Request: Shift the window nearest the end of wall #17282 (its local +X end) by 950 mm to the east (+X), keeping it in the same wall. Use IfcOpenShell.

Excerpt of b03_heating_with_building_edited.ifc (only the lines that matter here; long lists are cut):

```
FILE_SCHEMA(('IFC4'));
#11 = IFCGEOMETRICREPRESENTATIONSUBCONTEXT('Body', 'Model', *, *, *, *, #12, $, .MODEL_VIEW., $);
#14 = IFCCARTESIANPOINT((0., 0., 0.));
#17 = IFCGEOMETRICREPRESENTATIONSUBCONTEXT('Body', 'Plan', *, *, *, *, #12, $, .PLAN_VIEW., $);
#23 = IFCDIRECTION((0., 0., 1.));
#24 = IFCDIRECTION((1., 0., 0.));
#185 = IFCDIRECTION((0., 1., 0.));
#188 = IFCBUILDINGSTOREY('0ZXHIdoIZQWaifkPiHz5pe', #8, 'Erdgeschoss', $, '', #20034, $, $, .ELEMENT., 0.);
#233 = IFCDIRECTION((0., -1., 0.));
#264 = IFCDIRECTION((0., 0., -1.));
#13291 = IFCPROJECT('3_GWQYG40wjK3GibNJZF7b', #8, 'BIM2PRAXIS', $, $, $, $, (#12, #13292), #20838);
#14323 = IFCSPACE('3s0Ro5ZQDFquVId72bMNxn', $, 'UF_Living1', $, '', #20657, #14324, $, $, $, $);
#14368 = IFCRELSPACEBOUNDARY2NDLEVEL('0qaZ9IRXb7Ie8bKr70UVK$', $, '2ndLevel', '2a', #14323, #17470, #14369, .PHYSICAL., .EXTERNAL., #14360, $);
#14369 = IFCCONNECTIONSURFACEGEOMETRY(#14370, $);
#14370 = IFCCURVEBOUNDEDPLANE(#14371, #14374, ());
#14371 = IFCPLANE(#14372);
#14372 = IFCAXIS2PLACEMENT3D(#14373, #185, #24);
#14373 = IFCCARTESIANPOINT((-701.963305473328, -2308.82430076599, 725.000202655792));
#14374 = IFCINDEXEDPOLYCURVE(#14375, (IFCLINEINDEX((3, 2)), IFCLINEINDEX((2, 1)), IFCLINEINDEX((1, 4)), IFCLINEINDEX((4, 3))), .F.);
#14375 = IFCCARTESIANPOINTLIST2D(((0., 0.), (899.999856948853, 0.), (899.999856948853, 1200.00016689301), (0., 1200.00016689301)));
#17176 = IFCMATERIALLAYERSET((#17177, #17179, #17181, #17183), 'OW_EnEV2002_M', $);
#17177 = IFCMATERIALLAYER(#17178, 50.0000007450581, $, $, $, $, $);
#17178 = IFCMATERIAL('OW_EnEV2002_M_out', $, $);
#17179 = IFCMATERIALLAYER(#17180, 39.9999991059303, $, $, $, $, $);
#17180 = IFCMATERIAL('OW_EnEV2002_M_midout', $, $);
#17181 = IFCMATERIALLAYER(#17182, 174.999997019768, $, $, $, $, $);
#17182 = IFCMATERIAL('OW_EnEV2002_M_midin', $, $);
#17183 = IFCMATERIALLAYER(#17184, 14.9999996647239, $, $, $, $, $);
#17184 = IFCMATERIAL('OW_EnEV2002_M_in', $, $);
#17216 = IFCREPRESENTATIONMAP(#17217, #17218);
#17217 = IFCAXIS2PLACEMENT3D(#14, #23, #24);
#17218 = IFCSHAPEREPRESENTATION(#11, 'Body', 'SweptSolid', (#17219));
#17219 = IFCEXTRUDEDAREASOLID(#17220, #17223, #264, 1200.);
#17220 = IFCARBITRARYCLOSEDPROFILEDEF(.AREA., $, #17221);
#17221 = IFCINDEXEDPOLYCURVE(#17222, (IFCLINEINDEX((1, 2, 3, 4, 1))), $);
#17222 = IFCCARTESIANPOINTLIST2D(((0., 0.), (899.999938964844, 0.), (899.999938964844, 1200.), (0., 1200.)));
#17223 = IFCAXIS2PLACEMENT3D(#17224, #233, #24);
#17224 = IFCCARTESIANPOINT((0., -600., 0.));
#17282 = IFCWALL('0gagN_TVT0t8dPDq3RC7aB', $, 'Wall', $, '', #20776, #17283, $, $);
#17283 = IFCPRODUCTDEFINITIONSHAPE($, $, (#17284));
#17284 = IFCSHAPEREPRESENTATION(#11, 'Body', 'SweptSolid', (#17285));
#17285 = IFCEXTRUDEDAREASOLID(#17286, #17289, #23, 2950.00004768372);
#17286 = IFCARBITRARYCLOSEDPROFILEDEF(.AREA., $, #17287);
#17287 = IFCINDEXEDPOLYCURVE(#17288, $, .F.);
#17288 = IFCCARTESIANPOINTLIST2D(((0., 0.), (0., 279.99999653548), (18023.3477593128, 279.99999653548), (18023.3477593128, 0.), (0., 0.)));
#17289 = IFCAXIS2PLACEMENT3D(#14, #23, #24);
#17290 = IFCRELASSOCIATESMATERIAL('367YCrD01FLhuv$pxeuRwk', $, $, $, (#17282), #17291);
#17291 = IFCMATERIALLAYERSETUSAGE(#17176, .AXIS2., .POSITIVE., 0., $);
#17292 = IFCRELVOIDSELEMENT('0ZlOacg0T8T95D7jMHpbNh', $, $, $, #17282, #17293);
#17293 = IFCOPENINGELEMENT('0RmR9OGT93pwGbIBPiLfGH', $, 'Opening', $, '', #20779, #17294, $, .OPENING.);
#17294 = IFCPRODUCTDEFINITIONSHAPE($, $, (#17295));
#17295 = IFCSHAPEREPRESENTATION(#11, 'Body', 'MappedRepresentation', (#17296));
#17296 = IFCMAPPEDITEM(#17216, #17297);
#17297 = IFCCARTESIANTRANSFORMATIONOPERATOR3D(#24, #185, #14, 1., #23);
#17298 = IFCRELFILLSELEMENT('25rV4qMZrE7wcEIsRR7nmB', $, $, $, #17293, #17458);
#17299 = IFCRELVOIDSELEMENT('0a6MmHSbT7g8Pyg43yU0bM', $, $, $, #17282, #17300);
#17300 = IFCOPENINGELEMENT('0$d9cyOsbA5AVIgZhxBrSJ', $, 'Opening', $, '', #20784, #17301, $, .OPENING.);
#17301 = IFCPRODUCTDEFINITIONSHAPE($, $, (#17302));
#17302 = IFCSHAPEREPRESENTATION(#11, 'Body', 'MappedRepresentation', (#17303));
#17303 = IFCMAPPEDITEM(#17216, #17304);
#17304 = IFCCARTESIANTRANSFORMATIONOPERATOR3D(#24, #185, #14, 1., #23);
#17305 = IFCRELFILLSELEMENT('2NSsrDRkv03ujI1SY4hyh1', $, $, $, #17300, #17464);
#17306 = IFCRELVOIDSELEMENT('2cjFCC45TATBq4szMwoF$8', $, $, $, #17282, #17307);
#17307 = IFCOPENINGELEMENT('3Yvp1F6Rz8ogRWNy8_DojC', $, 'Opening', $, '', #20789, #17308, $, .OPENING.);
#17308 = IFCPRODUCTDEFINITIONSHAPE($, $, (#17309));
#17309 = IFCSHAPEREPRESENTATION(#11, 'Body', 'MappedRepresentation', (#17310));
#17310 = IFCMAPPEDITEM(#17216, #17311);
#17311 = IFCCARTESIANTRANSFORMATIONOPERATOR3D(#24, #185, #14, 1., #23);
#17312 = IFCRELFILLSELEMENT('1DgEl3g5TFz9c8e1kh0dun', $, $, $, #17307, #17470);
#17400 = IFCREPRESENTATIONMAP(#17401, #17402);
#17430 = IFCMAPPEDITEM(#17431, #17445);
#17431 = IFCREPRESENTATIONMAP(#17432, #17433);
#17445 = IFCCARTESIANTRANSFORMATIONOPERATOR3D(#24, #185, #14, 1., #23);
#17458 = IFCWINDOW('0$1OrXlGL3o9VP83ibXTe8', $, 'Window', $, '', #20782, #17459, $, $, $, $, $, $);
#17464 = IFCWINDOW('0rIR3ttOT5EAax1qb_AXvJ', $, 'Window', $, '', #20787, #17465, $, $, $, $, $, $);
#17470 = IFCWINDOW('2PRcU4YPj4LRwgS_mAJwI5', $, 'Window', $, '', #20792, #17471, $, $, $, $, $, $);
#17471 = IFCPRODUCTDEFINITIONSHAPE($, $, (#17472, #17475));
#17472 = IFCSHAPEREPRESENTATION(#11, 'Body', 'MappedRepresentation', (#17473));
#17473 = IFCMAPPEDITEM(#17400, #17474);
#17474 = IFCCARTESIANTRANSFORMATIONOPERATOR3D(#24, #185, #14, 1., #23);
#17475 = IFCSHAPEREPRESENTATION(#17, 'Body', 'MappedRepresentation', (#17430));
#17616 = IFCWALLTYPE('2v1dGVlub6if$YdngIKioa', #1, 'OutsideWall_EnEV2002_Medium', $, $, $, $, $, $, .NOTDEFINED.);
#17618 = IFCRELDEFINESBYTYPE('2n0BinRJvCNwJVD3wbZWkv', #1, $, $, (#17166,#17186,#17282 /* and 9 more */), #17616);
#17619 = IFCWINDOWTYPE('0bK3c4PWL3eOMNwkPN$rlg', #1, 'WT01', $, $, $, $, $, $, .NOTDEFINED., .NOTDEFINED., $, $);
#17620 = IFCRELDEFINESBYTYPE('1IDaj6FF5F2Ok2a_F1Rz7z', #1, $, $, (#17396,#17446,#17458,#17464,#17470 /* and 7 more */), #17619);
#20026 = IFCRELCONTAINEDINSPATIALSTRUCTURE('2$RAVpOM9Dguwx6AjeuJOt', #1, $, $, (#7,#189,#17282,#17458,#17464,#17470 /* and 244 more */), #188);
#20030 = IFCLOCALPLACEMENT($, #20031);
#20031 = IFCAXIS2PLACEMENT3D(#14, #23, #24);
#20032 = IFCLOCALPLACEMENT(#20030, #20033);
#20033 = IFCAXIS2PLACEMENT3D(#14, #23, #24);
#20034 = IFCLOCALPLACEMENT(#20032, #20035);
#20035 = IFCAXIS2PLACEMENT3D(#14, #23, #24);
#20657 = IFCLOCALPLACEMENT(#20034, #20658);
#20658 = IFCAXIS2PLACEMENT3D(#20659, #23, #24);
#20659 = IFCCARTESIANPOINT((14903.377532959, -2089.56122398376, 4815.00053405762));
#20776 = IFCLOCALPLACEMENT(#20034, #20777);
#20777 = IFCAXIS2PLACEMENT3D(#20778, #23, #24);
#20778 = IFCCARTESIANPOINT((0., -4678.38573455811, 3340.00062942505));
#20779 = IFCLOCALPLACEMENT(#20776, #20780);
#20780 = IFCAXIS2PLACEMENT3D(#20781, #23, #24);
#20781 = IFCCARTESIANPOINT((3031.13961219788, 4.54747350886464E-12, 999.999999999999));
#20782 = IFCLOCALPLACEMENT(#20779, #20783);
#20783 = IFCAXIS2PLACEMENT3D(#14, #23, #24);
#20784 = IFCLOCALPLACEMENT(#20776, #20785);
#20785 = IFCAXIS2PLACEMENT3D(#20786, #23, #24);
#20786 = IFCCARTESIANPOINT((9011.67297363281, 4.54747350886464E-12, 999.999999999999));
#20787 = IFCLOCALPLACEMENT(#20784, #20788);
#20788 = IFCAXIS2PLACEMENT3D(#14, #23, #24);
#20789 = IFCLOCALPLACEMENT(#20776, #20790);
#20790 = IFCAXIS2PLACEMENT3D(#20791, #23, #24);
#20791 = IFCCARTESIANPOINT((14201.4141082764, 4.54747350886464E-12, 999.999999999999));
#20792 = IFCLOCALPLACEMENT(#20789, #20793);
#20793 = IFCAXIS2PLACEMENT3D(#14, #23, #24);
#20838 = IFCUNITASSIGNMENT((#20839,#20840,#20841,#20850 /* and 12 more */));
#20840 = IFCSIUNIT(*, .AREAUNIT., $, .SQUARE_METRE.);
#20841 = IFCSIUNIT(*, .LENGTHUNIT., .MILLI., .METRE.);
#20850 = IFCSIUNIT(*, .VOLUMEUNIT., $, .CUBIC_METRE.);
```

```python
import numpy as np
import ifcopenshell
import ifcopenshell.api.geometry
import ifcopenshell.util.placement

model = ifcopenshell.open("b03_heating_with_building_edited.ifc")

window = model.by_guid("2PRcU4YPj4LRwgS_mAJwI5")
opening = window.FillsVoids[0].RelatingOpeningElement
wall = opening.VoidsElements[0].RelatingBuildingElement

wall_matrix = ifcopenshell.util.placement.get_local_placement(wall.ObjectPlacement)
shift = wall_matrix[:3, 0] * 950.0
before = ifcopenshell.util.placement.get_local_placement(window.ObjectPlacement)[:3, 3].copy()

# The window is placed relative to its opening, so it follows when the opening moves.
matrix = ifcopenshell.util.placement.get_local_placement(opening.ObjectPlacement)
matrix[:3, 3] += shift
ifcopenshell.api.geometry.edit_object_placement(
    model, product=opening, matrix=matrix, is_si=False, should_transform_children=True
)

# Space boundary surfaces are stored in each space's coordinates; move them too.
for rel in window.ProvidesBoundaries:
    if not rel.ConnectionGeometry:
        continue
    surface = rel.ConnectionGeometry.SurfaceOnRelatingElement.BasisSurface
    space_matrix = ifcopenshell.util.placement.get_local_placement(rel.RelatingSpace.ObjectPlacement)
    point = np.array(surface.Position.Location.Coordinates) + space_matrix[:3, :3].T @ shift
    surface.Position = model.createIfcAxis2Placement3D(
        model.createIfcCartesianPoint(point.tolist()), surface.Position.Axis, surface.Position.RefDirection
    )

after = ifcopenshell.util.placement.get_local_placement(window.ObjectPlacement)[:3, 3]
print("window moved by", (after - before).round(3) + 0.0)

model.write("b03_heating_with_building_edited_updated.ifc")
```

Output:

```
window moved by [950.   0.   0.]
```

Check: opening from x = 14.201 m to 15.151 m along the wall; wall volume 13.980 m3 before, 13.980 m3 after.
